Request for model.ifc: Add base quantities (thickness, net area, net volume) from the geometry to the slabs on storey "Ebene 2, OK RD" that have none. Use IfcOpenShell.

First a look at what the model holds.

```python
import ifcopenshell
import ifcopenshell.util.element
import ifcopenshell.util.unit

model = ifcopenshell.open("model.ifc")
print(model.schema)
for unit_type in ("LENGTHUNIT", "AREAUNIT", "VOLUMEUNIT"):
    print(unit_type, ifcopenshell.util.unit.calculate_unit_scale(model, unit_type))
storey = next(s for s in model.by_type("IfcBuildingStorey") if s.Name == "Ebene 2, OK RD")
slabs = [e for e in ifcopenshell.util.element.get_decomposition(storey) if e.is_a("IfcSlab")]
for e in sorted(slabs, key=lambda e: e.id()):
    print(e.id(), e.is_a(), e.Name, list(ifcopenshell.util.element.get_psets(e, qtos_only=True)), sep=" | ")
```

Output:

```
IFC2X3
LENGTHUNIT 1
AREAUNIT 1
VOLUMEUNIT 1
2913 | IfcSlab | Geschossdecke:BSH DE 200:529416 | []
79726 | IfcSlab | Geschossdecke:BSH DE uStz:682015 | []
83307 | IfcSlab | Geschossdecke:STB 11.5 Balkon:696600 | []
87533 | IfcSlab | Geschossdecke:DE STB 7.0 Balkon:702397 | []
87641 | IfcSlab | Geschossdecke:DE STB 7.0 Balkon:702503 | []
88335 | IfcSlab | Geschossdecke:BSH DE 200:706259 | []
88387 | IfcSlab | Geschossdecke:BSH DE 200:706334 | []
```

```python
import ifcopenshell
import ifcopenshell.api.pset
import ifcopenshell.geom
import ifcopenshell.util.element
import ifcopenshell.util.shape
import ifcopenshell.util.unit

model = ifcopenshell.open("model.ifc")
unit_scale = ifcopenshell.util.unit.calculate_unit_scale(model)
area_scale = ifcopenshell.util.unit.calculate_unit_scale(model, "AREAUNIT")
volume_scale = ifcopenshell.util.unit.calculate_unit_scale(model, "VOLUMEUNIT")
settings = ifcopenshell.geom.settings()

storey = next(s for s in model.by_type("IfcBuildingStorey") if s.Name == "Ebene 2, OK RD")
slabs = [e for e in ifcopenshell.util.element.get_decomposition(storey) if e.is_a("IfcSlab")]

for e in sorted(slabs, key=lambda e: e.id()):
    if ifcopenshell.util.element.get_psets(e, qtos_only=True, should_inherit=False):
        continue
    # Geometry comes back in metres, in the element's own axes.
    shape = ifcopenshell.geom.create_shape(settings, e)
    values = {
        "Width": ifcopenshell.util.shape.get_z(shape.geometry) / unit_scale,
        "NetArea": ifcopenshell.util.shape.get_footprint_area(shape.geometry) / area_scale,
        "NetVolume": ifcopenshell.util.shape.get_volume(shape.geometry) / volume_scale,
    }
    qto = ifcopenshell.api.pset.add_qto(model, product=e, name="BaseQuantities")
    ifcopenshell.api.pset.edit_qto(model, qto=qto, properties=values)
    print(e.id(), {k: round(v, 3) for k, v in values.items()})

model.write("model_rev.ifc")
```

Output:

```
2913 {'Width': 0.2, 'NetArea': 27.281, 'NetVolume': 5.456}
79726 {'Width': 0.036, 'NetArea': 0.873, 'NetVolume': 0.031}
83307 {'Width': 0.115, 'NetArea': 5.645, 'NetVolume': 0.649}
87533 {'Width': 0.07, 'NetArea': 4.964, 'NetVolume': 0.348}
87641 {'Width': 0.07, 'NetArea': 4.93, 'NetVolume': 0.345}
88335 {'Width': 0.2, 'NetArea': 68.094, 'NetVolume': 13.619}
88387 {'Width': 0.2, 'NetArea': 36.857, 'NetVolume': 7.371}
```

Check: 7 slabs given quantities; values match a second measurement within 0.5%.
